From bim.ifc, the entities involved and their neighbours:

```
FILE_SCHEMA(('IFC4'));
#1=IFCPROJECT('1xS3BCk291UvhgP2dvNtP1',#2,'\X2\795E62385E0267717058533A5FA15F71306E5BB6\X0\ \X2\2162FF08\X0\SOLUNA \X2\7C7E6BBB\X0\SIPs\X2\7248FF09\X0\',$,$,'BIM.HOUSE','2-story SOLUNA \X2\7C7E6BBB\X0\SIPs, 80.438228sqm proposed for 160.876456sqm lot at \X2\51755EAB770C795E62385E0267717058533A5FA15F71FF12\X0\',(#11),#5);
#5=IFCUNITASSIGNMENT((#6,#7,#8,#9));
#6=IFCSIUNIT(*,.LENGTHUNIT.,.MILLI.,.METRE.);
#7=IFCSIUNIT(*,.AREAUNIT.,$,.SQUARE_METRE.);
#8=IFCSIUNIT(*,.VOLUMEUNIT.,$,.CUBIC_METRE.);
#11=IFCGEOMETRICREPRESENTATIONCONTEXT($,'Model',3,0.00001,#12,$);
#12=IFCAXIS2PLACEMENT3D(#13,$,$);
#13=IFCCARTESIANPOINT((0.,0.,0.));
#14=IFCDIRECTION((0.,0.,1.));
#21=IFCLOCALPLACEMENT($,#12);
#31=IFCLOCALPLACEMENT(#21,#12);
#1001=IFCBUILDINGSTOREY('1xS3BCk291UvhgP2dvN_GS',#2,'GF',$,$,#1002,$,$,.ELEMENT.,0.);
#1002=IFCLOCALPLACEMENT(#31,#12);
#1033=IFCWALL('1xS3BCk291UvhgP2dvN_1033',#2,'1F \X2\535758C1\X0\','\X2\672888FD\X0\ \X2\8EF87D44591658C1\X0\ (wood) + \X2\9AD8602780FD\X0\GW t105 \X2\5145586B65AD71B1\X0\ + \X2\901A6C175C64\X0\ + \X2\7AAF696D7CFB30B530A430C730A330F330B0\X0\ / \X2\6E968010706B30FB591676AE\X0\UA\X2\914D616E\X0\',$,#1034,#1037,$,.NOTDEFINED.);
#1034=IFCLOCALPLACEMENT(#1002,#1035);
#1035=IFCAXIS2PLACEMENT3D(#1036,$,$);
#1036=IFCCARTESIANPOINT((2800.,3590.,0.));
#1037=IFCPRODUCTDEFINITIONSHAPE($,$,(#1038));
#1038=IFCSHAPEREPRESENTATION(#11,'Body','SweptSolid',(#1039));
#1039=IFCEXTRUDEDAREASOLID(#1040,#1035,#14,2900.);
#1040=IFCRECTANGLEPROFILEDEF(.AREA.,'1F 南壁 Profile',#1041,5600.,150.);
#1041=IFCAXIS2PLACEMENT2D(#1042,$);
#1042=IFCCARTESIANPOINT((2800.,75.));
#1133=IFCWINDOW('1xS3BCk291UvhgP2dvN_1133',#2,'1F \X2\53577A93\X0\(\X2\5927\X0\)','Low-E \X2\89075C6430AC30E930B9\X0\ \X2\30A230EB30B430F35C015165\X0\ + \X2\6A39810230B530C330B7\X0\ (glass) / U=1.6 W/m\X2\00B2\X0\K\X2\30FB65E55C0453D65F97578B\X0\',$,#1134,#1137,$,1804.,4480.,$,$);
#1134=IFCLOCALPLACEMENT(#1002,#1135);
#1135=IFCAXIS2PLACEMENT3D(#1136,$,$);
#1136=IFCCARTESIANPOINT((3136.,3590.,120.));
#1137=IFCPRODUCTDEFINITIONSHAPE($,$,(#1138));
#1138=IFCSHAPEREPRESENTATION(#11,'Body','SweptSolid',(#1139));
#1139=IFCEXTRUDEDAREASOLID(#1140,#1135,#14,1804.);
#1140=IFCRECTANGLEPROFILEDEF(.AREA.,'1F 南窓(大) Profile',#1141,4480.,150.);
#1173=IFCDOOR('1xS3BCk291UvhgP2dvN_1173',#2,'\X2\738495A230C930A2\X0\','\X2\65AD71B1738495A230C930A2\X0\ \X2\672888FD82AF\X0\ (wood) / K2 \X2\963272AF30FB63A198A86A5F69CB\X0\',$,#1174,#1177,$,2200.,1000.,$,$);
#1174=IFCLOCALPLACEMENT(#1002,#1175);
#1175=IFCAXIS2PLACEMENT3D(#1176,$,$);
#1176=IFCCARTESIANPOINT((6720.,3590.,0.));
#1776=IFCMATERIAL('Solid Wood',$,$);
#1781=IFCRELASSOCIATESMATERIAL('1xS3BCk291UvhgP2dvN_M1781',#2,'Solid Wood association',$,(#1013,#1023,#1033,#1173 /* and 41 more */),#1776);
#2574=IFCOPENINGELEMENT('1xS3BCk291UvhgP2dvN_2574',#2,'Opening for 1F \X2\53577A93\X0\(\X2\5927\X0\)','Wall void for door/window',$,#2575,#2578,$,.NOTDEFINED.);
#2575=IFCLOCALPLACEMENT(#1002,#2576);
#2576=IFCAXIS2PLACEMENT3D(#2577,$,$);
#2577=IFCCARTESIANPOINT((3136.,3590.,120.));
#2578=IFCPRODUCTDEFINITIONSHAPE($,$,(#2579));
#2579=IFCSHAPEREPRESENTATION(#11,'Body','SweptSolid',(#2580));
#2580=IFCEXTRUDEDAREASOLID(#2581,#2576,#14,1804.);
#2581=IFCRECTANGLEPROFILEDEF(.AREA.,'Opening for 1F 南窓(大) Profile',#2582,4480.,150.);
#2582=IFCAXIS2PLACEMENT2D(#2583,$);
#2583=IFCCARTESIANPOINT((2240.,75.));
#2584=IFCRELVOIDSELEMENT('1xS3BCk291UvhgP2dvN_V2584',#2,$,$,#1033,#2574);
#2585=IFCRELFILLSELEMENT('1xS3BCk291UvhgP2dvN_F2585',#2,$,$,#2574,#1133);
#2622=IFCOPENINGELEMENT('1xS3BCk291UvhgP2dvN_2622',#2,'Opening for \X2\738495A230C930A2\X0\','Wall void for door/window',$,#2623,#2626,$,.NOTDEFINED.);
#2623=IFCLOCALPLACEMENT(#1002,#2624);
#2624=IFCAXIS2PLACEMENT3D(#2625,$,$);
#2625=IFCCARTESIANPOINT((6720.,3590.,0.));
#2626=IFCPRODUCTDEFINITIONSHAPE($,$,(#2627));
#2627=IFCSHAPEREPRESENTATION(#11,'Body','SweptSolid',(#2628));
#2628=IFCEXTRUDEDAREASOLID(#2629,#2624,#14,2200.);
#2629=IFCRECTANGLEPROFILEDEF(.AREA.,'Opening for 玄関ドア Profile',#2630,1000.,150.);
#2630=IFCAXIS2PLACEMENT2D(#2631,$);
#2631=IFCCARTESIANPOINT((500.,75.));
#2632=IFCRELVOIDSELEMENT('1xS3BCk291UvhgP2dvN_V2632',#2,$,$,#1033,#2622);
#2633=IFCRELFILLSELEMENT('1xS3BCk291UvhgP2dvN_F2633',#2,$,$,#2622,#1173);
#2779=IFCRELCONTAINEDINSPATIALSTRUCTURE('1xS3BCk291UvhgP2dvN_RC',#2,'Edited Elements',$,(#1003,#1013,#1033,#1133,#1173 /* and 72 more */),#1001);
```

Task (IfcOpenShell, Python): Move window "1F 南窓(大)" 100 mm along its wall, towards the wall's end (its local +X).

```python
import ifcopenshell
import ifcopenshell.api.geometry
import ifcopenshell.util.placement
import ifcopenshell.util.unit

model = ifcopenshell.open("bim.ifc")
unit_scale = ifcopenshell.util.unit.calculate_unit_scale(model)

window = model.by_guid("1xS3BCk291UvhgP2dvN_1133")
opening = window.FillsVoids[0].RelatingOpeningElement
wall = opening.VoidsElements[0].RelatingBuildingElement

wall_matrix = ifcopenshell.util.placement.get_local_placement(wall.ObjectPlacement)
shift = wall_matrix[:3, 0] * 0.1 / unit_scale
before = ifcopenshell.util.placement.get_local_placement(window.ObjectPlacement)[:3, 3].copy()

# The window is not placed relative to its opening, so move both.
for product in (opening, window):
    matrix = ifcopenshell.util.placement.get_local_placement(product.ObjectPlacement)
    matrix[:3, 3] += shift
    ifcopenshell.api.geometry.edit_object_placement(model, product=product, matrix=matrix, is_si=False)

after = ifcopenshell.util.placement.get_local_placement(window.ObjectPlacement)[:3, 3]
print("window moved by", (after - before).round(3) + 0.0)

model.write("bim_edited.ifc")
```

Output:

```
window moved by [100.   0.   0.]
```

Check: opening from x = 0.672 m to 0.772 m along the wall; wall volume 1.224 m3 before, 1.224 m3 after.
